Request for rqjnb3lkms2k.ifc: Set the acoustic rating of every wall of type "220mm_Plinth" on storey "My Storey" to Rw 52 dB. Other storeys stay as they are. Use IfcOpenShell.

First a look at what the model holds.

```python
import ifcopenshell
import ifcopenshell.util.element

model = ifcopenshell.open("rqjnb3lkms2k.ifc")
print(model.schema)
storey = next(s for s in model.by_type("IfcBuildingStorey") if s.Name == "My Storey")
walls = [e for e in ifcopenshell.util.element.get_decomposition(storey) if e.is_a("IfcWall")]
seen = {}
for e in walls:
    element_type = ifcopenshell.util.element.get_type(e)
    key = (element_type.Name if element_type != e and element_type else None, ifcopenshell.util.element.get_pset(e, "Pset_WallCommon", "AcousticRating"))
    seen[key] = seen.get(key, 0) + 1
for (name, value), count in sorted(seen.items(), key=str):
    print(count, "x", name, "|", value)
```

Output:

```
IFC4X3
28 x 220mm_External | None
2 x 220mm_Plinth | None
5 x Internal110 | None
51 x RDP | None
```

```python
import ifcopenshell
import ifcopenshell.api.pset
import ifcopenshell.util.element

model = ifcopenshell.open("rqjnb3lkms2k.ifc")

storey = next(s for s in model.by_type("IfcBuildingStorey") if s.Name == "My Storey")
walls = [e for e in ifcopenshell.util.element.get_decomposition(storey) if e.is_a("IfcWall")]

count = 0
for e in walls:
    element_type = ifcopenshell.util.element.get_type(e)
    if element_type in (None, e) or element_type.Name != "220mm_Plinth":
        continue
    # add_pset returns the element's existing set when there is one.
    pset = ifcopenshell.api.pset.add_pset(model, product=e, name="Pset_WallCommon")
    ifcopenshell.api.pset.edit_pset(model, pset=pset, properties={"AcousticRating": "Rw 52 dB"})
    count += 1

print(count, "walls updated")

model.write("rqjnb3lkms2k_v2.ifc")
```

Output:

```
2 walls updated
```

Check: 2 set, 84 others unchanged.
